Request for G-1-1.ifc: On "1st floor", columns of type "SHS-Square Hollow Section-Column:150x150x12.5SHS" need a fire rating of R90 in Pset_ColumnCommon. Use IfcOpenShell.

First a look at what the model holds.

```python
import ifcopenshell
import ifcopenshell.util.element

model = ifcopenshell.open("G-1-1.ifc")
print(model.schema)
storey = next(s for s in model.by_type("IfcBuildingStorey") if s.Name == "1st floor")
columns = [e for e in ifcopenshell.util.element.get_decomposition(storey) if e.is_a("IfcColumn")]
seen = {}
for e in columns:
    element_type = ifcopenshell.util.element.get_type(e)
    key = (element_type.Name if element_type != e and element_type else None, ifcopenshell.util.element.get_pset(e, "Pset_ColumnCommon", "FireRating"))
    seen[key] = seen.get(key, 0) + 1
for (name, value), count in sorted(seen.items(), key=str):
    print(count, "x", name, "|", value)
```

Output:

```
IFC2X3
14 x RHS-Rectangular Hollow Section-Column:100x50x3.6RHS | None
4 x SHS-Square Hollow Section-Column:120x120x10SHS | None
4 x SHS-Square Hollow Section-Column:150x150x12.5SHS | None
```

```python
import ifcopenshell
import ifcopenshell.api.pset
import ifcopenshell.util.element

model = ifcopenshell.open("G-1-1.ifc")

storey = next(s for s in model.by_type("IfcBuildingStorey") if s.Name == "1st floor")
columns = [e for e in ifcopenshell.util.element.get_decomposition(storey) if e.is_a("IfcColumn")]

count = 0
for e in columns:
    element_type = ifcopenshell.util.element.get_type(e)
    if element_type in (None, e) or element_type.Name != "SHS-Square Hollow Section-Column:150x150x12.5SHS":
        continue
    # add_pset returns the element's existing set when there is one.
    pset = ifcopenshell.api.pset.add_pset(model, product=e, name="Pset_ColumnCommon")
    ifcopenshell.api.pset.edit_pset(model, pset=pset, properties={"FireRating": "R90"})
    count += 1

print(count, "columns updated")

model.write("G-1-1_edited.ifc")
```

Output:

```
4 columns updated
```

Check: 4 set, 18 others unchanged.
